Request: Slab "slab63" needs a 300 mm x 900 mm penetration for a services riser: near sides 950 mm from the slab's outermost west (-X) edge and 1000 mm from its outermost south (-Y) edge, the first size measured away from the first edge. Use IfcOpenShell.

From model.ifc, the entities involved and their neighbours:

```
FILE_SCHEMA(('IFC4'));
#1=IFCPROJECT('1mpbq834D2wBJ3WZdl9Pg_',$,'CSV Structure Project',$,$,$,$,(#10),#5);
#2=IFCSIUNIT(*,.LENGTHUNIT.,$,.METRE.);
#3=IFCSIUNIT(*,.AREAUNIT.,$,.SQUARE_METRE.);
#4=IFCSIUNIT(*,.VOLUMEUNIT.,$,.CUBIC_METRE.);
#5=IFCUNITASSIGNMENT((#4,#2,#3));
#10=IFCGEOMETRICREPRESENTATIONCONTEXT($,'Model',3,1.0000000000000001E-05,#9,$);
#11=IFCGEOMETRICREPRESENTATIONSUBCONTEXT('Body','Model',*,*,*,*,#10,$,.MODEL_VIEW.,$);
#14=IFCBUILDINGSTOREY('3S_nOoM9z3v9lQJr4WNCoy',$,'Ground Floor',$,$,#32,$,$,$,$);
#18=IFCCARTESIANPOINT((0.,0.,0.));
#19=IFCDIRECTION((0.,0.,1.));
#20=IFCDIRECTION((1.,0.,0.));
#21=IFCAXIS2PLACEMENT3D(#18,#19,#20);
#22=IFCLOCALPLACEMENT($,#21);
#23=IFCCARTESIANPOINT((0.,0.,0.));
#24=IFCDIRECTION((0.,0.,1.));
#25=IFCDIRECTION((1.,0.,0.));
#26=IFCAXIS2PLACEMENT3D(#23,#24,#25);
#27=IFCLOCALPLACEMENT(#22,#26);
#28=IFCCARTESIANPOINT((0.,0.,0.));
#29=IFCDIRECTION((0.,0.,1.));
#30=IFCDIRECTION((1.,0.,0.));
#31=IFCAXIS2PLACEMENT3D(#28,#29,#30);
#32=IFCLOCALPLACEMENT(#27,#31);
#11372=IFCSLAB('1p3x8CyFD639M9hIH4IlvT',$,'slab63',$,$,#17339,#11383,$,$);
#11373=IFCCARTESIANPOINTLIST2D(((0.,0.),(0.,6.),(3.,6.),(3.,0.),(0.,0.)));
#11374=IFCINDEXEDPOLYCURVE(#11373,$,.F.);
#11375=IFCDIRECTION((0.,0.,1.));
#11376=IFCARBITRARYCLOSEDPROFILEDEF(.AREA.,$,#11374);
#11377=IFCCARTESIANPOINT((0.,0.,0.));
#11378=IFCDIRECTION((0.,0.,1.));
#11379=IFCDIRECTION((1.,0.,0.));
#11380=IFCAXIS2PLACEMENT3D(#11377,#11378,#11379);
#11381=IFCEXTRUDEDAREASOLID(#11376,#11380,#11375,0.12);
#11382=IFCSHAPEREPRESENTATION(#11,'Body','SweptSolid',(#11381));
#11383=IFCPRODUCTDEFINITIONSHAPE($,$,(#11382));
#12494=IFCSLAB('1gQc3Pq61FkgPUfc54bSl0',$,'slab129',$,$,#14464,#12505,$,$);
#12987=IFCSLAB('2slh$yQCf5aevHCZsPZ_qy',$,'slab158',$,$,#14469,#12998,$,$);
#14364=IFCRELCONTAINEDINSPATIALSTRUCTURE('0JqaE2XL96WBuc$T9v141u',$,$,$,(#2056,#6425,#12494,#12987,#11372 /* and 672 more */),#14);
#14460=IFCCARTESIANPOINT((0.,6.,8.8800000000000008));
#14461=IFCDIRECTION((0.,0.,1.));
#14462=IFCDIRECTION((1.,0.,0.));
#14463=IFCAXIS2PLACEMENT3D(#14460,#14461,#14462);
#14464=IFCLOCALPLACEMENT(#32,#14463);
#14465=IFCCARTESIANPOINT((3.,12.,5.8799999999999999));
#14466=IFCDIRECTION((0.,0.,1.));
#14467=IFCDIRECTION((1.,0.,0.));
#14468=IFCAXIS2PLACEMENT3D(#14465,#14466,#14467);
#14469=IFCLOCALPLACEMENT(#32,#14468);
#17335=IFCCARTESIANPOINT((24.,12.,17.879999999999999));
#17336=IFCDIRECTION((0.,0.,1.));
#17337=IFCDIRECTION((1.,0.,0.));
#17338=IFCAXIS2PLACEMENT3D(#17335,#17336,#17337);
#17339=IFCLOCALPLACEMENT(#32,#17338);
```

```python
import numpy as np
import ifcopenshell
import ifcopenshell.api.feature
import ifcopenshell.api.geometry
import ifcopenshell.api.root
import ifcopenshell.geom
import ifcopenshell.util.placement
import ifcopenshell.util.representation
import ifcopenshell.util.shape
import ifcopenshell.util.unit

model = ifcopenshell.open("model.ifc")
unit_scale = ifcopenshell.util.unit.calculate_unit_scale(model)
settings = ifcopenshell.geom.settings()


def volume(element):
    """Net volume in cubic metres, openings subtracted."""
    shape = ifcopenshell.geom.create_shape(settings, element)
    return ifcopenshell.util.shape.get_volume(shape.geometry)


slab = model.by_guid("1p3x8CyFD639M9hIH4IlvT")
before = volume(slab)

# Extent in the slab's own axes, in metres. The edges named are its -X and -Y sides.
slab_shape = ifcopenshell.geom.create_shape(settings, slab)
vertices = ifcopenshell.util.shape.get_vertices(slab_shape.geometry)
x_min, y_min, bottom = vertices.min(axis=0)
top = vertices[:, 2].max()

opening = ifcopenshell.api.root.create_entity(model, ifc_class="IfcOpeningElement", name="Services riser opening", predefined_type="OPENING")
context = ifcopenshell.util.representation.get_context(model, "Model", "Body", "MODEL_VIEW")
width, depth = 0.3, 0.9
outline = [(0.0, 0.0), (width, 0.0), (width, depth), (0.0, depth), (0.0, 0.0)]
# Overshoot both faces by 50 mm so the cut is clean.
shape = ifcopenshell.api.geometry.add_slab_representation(
    model, context=context, depth=top - bottom + 0.1, polyline=outline
)
ifcopenshell.api.geometry.assign_representation(model, product=opening, representation=shape)

matrix = ifcopenshell.util.placement.get_local_placement(slab.ObjectPlacement)
matrix[:, 3] = matrix @ np.append(np.array([x_min + 0.95, y_min + 1, bottom - 0.05]) / unit_scale, 1.0)
ifcopenshell.api.geometry.edit_object_placement(model, product=opening, matrix=matrix, is_si=False)
ifcopenshell.api.feature.add_feature(model, feature=opening, element=slab)

after = volume(slab)

print(f"slab volume {before:.3f} -> {after:.3f} m3")

model.write("model_v2.ifc")
```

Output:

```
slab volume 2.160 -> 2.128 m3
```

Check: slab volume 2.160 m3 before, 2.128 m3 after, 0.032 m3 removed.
